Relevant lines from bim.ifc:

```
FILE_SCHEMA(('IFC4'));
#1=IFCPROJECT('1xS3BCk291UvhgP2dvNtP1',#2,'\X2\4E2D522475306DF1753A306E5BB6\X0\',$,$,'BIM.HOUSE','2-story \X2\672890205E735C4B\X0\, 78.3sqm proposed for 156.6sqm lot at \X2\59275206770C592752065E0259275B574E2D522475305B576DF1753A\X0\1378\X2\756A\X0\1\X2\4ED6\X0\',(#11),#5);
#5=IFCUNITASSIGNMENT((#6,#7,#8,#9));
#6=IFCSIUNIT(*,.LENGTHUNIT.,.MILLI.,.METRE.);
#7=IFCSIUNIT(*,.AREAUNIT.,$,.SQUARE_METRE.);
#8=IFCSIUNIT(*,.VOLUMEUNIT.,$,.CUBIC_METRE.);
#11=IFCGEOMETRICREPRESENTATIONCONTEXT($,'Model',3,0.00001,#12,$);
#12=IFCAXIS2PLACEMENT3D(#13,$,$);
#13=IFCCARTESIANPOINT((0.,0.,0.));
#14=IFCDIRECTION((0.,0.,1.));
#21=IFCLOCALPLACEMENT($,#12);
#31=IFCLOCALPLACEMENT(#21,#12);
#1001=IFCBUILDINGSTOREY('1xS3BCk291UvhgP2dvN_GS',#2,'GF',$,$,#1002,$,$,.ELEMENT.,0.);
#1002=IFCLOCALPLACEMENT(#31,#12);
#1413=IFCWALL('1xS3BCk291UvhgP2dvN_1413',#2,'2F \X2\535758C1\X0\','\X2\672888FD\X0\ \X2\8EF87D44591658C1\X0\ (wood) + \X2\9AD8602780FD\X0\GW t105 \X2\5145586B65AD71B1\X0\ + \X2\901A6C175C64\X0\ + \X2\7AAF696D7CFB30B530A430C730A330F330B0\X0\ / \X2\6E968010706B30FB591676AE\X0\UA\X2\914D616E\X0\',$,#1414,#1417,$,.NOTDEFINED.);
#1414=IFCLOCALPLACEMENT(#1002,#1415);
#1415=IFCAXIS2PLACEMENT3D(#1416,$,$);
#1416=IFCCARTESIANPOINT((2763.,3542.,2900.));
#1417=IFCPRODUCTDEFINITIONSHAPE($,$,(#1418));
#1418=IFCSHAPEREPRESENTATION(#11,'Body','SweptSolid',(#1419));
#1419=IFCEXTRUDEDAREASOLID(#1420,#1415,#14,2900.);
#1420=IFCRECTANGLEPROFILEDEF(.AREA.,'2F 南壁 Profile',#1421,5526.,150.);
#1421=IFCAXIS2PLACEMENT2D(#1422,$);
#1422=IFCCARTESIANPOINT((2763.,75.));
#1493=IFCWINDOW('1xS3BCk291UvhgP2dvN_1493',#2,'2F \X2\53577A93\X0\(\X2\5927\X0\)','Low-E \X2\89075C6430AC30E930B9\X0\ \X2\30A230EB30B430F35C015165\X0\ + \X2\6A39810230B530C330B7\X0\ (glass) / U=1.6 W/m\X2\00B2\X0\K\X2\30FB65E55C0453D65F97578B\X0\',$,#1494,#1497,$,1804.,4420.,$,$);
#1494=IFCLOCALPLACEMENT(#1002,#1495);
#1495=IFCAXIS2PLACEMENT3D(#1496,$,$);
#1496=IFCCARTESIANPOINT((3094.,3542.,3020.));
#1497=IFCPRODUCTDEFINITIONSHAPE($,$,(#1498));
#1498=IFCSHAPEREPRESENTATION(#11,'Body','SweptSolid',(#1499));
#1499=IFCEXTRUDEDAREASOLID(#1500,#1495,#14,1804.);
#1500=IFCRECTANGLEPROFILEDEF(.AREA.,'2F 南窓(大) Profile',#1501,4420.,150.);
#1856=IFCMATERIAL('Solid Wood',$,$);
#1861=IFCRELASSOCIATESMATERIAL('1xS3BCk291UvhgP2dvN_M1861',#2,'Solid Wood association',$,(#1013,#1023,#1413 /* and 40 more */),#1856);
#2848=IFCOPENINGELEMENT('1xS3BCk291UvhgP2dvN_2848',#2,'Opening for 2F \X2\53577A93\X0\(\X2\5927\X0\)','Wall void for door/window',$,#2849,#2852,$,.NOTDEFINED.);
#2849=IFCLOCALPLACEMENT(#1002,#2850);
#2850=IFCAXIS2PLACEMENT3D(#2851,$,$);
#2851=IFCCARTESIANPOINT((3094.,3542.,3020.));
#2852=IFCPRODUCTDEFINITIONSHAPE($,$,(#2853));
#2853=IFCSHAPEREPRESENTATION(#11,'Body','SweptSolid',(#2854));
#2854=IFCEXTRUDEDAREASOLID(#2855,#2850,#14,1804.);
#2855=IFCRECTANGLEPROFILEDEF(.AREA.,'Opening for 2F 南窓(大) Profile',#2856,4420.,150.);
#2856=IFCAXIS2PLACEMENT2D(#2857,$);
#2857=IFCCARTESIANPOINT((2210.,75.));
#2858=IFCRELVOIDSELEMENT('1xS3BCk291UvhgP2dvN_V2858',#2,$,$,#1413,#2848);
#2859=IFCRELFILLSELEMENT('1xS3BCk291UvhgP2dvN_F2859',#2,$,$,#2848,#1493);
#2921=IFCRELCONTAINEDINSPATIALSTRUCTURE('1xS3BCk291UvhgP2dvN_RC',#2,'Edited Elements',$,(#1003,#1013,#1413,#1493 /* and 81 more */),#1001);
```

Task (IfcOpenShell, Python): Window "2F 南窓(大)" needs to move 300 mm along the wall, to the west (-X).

```python
import ifcopenshell
import ifcopenshell.api.geometry
import ifcopenshell.util.placement

model = ifcopenshell.open("bim.ifc")

window = model.by_guid("1xS3BCk291UvhgP2dvN_1493")
opening = window.FillsVoids[0].RelatingOpeningElement
wall = opening.VoidsElements[0].RelatingBuildingElement

wall_matrix = ifcopenshell.util.placement.get_local_placement(wall.ObjectPlacement)
shift = wall_matrix[:3, 0] * -300.0
before = ifcopenshell.util.placement.get_local_placement(window.ObjectPlacement)[:3, 3].copy()

# The window is not placed relative to its opening, so move both.
for product in (opening, window):
    matrix = ifcopenshell.util.placement.get_local_placement(product.ObjectPlacement)
    matrix[:3, 3] += shift
    ifcopenshell.api.geometry.edit_object_placement(model, product=product, matrix=matrix, is_si=False)

after = ifcopenshell.util.placement.get_local_placement(window.ObjectPlacement)[:3, 3]
print("window moved by", (after - before).round(3) + 0.0)

model.write("bim_updated.ifc")
```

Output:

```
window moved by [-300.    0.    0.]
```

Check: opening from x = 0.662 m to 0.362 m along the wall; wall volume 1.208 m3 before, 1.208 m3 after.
